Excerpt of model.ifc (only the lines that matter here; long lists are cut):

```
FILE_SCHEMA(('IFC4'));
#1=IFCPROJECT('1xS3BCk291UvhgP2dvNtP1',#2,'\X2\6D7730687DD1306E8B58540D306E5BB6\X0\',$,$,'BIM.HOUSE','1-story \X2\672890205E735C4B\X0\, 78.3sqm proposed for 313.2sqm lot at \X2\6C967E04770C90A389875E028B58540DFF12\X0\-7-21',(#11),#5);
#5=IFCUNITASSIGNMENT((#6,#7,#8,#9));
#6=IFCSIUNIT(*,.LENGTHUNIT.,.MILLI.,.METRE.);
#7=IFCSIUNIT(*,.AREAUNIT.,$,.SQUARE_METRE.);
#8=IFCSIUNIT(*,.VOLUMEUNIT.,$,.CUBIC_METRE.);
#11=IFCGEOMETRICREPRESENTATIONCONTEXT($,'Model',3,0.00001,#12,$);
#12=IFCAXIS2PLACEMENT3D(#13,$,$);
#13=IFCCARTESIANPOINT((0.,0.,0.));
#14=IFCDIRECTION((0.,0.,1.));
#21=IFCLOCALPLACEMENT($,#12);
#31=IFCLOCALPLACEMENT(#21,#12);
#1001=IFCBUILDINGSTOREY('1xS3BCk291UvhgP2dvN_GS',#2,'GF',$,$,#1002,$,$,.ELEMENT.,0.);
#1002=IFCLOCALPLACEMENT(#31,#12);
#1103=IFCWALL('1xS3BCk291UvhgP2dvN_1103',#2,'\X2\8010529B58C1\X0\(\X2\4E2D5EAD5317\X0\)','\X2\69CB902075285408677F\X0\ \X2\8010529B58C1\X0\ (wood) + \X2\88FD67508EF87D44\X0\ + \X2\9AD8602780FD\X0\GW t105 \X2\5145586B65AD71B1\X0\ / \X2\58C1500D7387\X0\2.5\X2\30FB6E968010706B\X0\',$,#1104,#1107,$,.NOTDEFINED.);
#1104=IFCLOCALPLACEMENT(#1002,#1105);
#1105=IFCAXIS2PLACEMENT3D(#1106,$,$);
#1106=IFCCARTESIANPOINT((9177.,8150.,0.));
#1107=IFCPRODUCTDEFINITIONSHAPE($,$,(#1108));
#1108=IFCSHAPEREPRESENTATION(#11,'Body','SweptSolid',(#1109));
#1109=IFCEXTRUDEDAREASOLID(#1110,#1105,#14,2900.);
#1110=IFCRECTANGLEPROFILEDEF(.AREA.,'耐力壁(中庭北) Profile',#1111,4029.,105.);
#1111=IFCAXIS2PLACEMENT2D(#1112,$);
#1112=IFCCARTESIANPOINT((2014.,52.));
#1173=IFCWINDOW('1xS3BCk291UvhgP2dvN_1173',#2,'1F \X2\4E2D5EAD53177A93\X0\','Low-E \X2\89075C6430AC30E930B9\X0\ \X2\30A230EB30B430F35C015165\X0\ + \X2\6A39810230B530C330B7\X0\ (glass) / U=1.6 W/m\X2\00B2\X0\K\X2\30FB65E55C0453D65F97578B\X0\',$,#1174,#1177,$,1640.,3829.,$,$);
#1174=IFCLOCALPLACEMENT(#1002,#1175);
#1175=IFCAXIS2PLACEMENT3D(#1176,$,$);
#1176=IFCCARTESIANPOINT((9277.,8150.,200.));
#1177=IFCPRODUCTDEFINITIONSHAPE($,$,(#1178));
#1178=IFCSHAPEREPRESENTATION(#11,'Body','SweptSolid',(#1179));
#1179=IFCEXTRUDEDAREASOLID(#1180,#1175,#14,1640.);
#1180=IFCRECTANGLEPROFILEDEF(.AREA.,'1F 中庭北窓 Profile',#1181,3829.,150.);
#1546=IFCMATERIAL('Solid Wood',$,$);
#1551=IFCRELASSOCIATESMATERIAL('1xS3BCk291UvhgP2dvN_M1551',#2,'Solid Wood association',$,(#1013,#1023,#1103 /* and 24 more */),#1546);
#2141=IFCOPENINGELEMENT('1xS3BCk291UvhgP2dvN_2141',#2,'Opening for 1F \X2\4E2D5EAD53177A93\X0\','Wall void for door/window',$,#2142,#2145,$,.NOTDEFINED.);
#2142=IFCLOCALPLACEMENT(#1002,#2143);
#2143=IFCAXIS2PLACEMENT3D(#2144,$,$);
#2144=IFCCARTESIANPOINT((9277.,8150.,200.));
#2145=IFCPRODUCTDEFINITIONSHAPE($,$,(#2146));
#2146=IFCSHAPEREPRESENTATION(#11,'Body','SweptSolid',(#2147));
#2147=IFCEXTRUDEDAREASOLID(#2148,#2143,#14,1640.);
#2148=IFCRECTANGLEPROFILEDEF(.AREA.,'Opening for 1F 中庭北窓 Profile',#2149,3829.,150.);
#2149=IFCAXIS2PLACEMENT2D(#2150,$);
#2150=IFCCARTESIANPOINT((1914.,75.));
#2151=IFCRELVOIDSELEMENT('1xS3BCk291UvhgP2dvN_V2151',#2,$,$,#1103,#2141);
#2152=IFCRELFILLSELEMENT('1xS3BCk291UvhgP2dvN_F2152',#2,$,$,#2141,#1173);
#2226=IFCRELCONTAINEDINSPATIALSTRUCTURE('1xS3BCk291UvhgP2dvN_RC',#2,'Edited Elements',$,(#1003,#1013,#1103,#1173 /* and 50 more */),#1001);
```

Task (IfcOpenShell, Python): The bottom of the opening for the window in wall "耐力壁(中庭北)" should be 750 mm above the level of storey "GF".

```python
import numpy as np
import ifcopenshell
import ifcopenshell.api.geometry
import ifcopenshell.geom
import ifcopenshell.util.element
import ifcopenshell.util.placement
import ifcopenshell.util.shape
import ifcopenshell.util.unit

model = ifcopenshell.open("model.ifc")
unit_scale = ifcopenshell.util.unit.calculate_unit_scale(model)

window = model.by_guid("1xS3BCk291UvhgP2dvN_1173")
opening = window.FillsVoids[0].RelatingOpeningElement
storey = ifcopenshell.util.element.get_container(window, ifc_class="IfcBuildingStorey")
level = ifcopenshell.util.placement.get_local_placement(storey.ObjectPlacement)[2, 3]

# The opening's origin need not be at the sill, so measure its lowest point.
shape = ifcopenshell.geom.create_shape(ifcopenshell.geom.settings(), opening)
bottom = ifcopenshell.util.shape.get_shape_bottom_elevation(shape, shape.geometry) / unit_scale
dz = level + 0.75 / unit_scale - bottom

shift = np.array([0.0, 0.0, dz])
# The window is not placed relative to its opening, so move both.
for product in (opening, window):
    matrix = ifcopenshell.util.placement.get_local_placement(product.ObjectPlacement)
    matrix[:3, 3] += shift
    ifcopenshell.api.geometry.edit_object_placement(model, product=product, matrix=matrix, is_si=False)

print(f"moved by {dz * unit_scale:+.3f} m")

model.write("model_updated.ifc")
```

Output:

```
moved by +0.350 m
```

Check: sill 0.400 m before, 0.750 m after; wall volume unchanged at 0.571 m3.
